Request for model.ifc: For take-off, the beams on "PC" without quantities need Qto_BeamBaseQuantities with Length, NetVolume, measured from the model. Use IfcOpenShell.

First a look at what the model holds.

```python
import ifcopenshell
import ifcopenshell.util.element
import ifcopenshell.util.unit

model = ifcopenshell.open("model.ifc")
print(model.schema)
for unit_type in ("LENGTHUNIT", "AREAUNIT", "VOLUMEUNIT"):
    print(unit_type, ifcopenshell.util.unit.calculate_unit_scale(model, unit_type))
storey = next(s for s in model.by_type("IfcBuildingStorey") if s.Name == "PC")
beams = [e for e in ifcopenshell.util.element.get_decomposition(storey) if e.is_a("IfcBeam")]
for e in sorted(beams, key=lambda e: e.id()):
    print(e.id(), e.is_a(), e.Name, list(ifcopenshell.util.element.get_psets(e, qtos_only=True)), sep=" | ")
```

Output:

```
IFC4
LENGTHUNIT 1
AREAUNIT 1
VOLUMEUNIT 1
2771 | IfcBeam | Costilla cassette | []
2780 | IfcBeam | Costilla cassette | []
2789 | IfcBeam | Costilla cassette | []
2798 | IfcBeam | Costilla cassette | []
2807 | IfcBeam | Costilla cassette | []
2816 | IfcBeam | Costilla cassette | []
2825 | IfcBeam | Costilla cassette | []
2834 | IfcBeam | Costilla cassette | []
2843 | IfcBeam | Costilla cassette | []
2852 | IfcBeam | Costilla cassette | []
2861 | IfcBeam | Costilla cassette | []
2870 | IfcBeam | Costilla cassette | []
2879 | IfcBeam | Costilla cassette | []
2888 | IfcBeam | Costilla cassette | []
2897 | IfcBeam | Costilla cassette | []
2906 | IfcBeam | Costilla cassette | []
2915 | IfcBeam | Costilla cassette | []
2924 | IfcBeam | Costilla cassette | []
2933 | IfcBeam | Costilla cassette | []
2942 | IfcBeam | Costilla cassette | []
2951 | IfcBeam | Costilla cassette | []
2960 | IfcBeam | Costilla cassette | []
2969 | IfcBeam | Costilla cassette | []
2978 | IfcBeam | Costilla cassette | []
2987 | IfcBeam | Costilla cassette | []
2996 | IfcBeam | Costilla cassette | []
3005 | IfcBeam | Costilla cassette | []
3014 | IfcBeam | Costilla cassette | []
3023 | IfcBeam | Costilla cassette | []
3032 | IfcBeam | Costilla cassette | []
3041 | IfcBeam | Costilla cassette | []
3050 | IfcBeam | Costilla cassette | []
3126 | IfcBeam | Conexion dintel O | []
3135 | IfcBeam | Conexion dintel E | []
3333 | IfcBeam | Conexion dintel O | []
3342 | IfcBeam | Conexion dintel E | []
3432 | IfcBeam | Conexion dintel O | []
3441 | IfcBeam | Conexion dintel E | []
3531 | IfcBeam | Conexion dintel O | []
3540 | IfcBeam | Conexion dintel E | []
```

```python
import ifcopenshell
import ifcopenshell.api.pset
import ifcopenshell.geom
import ifcopenshell.util.element
import ifcopenshell.util.shape
import ifcopenshell.util.unit

model = ifcopenshell.open("model.ifc")
unit_scale = ifcopenshell.util.unit.calculate_unit_scale(model)
volume_scale = ifcopenshell.util.unit.calculate_unit_scale(model, "VOLUMEUNIT")
settings = ifcopenshell.geom.settings()

storey = next(s for s in model.by_type("IfcBuildingStorey") if s.Name == "PC")
beams = [e for e in ifcopenshell.util.element.get_decomposition(storey) if e.is_a("IfcBeam")]

for e in sorted(beams, key=lambda e: e.id()):
    if ifcopenshell.util.element.get_psets(e, qtos_only=True, should_inherit=False):
        continue
    # Geometry comes back in metres, in the element's own axes.
    shape = ifcopenshell.geom.create_shape(settings, e)
    values = {
        "Length": ifcopenshell.util.shape.get_max_xyz(shape.geometry) / unit_scale,
        "NetVolume": ifcopenshell.util.shape.get_volume(shape.geometry) / volume_scale,
    }
    qto = ifcopenshell.api.pset.add_qto(model, product=e, name="Qto_BeamBaseQuantities")
    ifcopenshell.api.pset.edit_qto(model, qto=qto, properties=values)
    print(e.id(), {k: round(v, 3) for k, v in values.items()})

model.write("model_v2.ifc")
```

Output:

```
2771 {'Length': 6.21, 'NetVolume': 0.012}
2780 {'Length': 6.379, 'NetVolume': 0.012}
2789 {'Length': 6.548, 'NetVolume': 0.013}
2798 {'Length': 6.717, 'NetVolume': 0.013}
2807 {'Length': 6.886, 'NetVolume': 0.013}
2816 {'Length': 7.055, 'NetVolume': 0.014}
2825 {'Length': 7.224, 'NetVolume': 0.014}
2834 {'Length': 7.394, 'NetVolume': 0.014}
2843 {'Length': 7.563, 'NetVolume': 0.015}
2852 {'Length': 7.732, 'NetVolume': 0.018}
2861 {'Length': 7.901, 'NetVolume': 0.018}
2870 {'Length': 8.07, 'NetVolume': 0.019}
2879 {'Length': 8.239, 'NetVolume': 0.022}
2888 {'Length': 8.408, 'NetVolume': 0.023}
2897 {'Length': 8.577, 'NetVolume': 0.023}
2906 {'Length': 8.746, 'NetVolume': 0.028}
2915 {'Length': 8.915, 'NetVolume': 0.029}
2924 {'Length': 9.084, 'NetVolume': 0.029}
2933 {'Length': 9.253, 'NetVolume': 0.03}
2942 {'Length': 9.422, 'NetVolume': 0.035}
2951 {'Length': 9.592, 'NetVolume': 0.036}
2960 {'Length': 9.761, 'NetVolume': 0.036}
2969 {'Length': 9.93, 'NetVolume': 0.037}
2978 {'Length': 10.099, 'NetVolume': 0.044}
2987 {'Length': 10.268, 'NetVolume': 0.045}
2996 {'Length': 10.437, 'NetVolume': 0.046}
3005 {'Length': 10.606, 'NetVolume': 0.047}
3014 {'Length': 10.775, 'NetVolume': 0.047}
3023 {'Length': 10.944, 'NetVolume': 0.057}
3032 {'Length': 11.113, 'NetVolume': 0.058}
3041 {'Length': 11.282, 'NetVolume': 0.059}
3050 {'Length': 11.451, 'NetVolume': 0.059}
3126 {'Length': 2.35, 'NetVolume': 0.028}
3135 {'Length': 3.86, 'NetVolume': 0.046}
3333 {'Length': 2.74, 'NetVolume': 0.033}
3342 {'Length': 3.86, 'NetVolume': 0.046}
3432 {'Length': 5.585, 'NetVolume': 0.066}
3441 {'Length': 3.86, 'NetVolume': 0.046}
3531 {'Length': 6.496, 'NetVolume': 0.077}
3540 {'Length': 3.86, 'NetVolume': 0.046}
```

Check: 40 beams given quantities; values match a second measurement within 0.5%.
